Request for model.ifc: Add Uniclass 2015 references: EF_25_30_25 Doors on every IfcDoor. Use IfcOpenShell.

First a look at what the model holds.

```python
import ifcopenshell

model = ifcopenshell.open("model.ifc")
print(model.schema)
print("classifications:", [c.Name for c in model.by_type("IfcClassification")])
for ifc_class in ("IfcDoor", "IfcRoof", "IfcStair", "IfcWall", "IfcWindow"):
    print(ifc_class, len(model.by_type(ifc_class)))
```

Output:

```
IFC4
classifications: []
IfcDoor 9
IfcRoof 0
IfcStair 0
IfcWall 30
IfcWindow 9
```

```python
import ifcopenshell
import ifcopenshell.api.classification

model = ifcopenshell.open("model.ifc")

system = ifcopenshell.api.classification.add_classification(model, classification="Uniclass 2015")

codes = {
    "IfcDoor": ("EF_25_30_25", "Doors"),
}
for ifc_class, (code, name) in codes.items():
    products = model.by_type(ifc_class)
    ifcopenshell.api.classification.add_reference(
        model, products=products, classification=system, identification=code, name=name
    )
    print(code, len(products))

model.write("model_updated.ifc")
```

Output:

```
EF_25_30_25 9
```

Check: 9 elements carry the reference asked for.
